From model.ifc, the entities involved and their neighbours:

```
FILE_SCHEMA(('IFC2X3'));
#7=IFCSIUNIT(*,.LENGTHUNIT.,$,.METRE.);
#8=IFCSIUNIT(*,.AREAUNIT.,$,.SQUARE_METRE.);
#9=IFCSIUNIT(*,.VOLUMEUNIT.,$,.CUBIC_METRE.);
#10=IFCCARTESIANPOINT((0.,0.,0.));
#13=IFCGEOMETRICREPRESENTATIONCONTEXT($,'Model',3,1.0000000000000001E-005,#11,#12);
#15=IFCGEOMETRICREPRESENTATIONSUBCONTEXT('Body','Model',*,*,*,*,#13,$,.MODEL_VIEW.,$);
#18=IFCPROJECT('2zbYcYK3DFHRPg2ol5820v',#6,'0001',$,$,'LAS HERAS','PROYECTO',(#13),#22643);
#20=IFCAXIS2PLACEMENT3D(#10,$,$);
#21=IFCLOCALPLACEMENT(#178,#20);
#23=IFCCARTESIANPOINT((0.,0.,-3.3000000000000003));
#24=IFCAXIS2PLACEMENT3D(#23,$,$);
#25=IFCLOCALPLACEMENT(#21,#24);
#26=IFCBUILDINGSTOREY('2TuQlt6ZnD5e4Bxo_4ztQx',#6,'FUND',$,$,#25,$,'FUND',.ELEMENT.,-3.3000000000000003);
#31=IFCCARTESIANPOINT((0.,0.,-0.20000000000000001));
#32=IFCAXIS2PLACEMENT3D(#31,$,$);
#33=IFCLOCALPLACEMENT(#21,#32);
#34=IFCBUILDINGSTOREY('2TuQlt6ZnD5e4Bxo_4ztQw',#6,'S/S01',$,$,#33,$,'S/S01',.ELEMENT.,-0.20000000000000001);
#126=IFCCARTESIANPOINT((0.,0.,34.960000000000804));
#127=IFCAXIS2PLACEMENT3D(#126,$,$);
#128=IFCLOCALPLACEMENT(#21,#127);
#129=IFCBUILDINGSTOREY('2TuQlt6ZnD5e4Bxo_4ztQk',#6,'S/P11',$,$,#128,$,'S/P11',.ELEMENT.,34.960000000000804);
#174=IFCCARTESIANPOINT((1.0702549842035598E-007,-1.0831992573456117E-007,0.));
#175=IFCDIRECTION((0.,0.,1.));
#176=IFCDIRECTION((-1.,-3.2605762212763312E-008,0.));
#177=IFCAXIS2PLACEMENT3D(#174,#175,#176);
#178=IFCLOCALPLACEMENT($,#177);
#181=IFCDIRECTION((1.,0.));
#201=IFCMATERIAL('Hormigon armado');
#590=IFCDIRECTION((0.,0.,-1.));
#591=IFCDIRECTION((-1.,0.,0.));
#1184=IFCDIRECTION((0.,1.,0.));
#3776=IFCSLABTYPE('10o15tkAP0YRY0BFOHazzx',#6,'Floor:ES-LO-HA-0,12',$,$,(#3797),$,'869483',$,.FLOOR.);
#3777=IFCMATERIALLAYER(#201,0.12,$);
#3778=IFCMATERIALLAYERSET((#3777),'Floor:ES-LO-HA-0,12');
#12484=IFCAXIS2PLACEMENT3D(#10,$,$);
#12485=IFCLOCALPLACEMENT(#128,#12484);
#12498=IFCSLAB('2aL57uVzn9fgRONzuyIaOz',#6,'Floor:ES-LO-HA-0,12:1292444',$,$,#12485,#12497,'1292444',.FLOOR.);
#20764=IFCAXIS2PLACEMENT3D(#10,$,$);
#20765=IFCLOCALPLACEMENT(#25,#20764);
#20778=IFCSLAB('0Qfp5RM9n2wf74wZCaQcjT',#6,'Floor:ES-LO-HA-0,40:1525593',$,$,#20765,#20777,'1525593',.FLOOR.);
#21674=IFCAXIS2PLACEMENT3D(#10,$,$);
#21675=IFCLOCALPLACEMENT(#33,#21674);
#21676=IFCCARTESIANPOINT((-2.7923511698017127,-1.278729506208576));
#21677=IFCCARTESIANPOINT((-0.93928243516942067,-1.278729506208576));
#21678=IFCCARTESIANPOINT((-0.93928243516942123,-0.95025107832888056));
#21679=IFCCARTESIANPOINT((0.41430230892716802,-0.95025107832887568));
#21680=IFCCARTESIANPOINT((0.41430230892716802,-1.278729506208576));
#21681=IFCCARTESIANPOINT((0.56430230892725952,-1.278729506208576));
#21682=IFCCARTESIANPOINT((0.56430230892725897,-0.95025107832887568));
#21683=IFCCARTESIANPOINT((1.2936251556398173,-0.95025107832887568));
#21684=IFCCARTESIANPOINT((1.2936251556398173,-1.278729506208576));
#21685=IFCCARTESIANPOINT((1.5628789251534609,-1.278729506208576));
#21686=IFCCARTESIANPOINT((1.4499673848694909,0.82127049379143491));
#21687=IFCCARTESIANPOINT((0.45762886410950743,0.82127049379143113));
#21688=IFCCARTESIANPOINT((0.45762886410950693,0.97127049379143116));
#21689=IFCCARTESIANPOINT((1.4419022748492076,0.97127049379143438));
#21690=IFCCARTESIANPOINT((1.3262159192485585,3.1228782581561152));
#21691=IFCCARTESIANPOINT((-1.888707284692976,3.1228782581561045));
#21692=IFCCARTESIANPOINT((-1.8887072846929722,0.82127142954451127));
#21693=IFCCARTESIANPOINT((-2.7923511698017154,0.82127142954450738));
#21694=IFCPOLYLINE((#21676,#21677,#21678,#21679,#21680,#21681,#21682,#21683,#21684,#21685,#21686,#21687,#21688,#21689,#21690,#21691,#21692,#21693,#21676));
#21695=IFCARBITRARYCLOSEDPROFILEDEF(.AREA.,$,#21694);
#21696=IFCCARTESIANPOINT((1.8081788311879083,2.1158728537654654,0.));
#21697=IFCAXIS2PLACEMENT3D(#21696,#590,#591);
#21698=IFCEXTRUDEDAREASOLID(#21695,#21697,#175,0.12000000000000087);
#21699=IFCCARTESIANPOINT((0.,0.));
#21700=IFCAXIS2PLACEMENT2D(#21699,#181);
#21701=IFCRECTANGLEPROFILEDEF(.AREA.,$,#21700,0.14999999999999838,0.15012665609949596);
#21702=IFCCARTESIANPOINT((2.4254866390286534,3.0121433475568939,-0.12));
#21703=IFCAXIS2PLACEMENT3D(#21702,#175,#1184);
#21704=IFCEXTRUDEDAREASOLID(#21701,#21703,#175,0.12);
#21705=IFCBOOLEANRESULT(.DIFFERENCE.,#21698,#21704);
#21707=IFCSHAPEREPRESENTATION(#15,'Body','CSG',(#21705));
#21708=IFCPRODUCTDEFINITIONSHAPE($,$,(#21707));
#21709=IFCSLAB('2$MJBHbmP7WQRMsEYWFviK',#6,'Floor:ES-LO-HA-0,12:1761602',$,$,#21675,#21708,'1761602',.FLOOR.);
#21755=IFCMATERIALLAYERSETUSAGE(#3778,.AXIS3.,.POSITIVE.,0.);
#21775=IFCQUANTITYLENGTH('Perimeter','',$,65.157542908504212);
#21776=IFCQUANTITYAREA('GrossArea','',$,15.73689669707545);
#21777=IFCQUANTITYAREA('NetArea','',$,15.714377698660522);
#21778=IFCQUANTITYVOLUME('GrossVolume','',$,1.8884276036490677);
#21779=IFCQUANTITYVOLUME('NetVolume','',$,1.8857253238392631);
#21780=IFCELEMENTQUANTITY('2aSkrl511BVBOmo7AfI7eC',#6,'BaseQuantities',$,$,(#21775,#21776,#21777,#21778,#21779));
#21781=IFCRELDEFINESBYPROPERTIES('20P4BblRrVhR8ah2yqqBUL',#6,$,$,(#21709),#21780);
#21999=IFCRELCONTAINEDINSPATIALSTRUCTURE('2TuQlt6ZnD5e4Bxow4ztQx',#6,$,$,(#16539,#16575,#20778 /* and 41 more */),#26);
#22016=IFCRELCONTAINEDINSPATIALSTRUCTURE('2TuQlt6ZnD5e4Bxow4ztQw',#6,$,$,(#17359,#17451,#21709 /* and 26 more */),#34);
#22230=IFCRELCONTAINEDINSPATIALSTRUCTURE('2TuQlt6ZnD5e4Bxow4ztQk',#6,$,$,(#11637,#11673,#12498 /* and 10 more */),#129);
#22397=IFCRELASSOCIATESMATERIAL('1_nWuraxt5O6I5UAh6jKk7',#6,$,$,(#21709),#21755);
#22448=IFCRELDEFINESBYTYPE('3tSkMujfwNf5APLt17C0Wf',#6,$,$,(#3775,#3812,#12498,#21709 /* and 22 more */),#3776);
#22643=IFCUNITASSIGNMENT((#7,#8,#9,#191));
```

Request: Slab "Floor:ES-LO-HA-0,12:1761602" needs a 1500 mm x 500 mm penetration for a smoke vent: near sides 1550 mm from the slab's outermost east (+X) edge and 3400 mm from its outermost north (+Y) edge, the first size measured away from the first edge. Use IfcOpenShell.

```python
import numpy as np
import ifcopenshell
import ifcopenshell.api.feature
import ifcopenshell.api.geometry
import ifcopenshell.api.pset
import ifcopenshell.api.root
import ifcopenshell.geom
import ifcopenshell.util.element
import ifcopenshell.util.placement
import ifcopenshell.util.representation
import ifcopenshell.util.shape
import ifcopenshell.util.unit

model = ifcopenshell.open("model.ifc")
unit_scale = ifcopenshell.util.unit.calculate_unit_scale(model)
area_scale = ifcopenshell.util.unit.calculate_unit_scale(model, "AREAUNIT")
volume_scale = ifcopenshell.util.unit.calculate_unit_scale(model, "VOLUMEUNIT")
settings = ifcopenshell.geom.settings()


def volume(element):
    """Net volume in cubic metres, openings subtracted."""
    shape = ifcopenshell.geom.create_shape(settings, element)
    return ifcopenshell.util.shape.get_volume(shape.geometry)


slab = model.by_guid("2$MJBHbmP7WQRMsEYWFviK")
before = volume(slab)

# Extent in the slab's own axes, in metres. The edges named are its -X and -Y sides.
slab_shape = ifcopenshell.geom.create_shape(settings, slab)
vertices = ifcopenshell.util.shape.get_vertices(slab_shape.geometry)
x_min, y_min, bottom = vertices.min(axis=0)
top = vertices[:, 2].max()

opening = ifcopenshell.api.root.create_entity(model, ifc_class="IfcOpeningElement", name="Smoke vent opening")
context = ifcopenshell.util.representation.get_context(model, "Model", "Body", "MODEL_VIEW")
width, depth = 1.5, 0.5
outline = [(0.0, 0.0), (width, 0.0), (width, depth), (0.0, depth), (0.0, 0.0)]
# Overshoot both faces by 50 mm so the cut is clean.
shape = ifcopenshell.api.geometry.add_slab_representation(
    model, context=context, depth=top - bottom + 0.1, polyline=outline
)
ifcopenshell.api.geometry.assign_representation(model, product=opening, representation=shape)

matrix = ifcopenshell.util.placement.get_local_placement(slab.ObjectPlacement)
matrix[:, 3] = matrix @ np.append(np.array([x_min + 1.55, y_min + 3.4, bottom - 0.05]) / unit_scale, 1.0)
ifcopenshell.api.geometry.edit_object_placement(model, product=opening, matrix=matrix, is_si=False)
ifcopenshell.api.feature.add_feature(model, feature=opening, element=slab)

after = volume(slab)

# Update the slab's stored quantities.
qto = model.by_id(ifcopenshell.util.element.get_pset(slab, "BaseQuantities", should_inherit=False)["id"])
ifcopenshell.api.pset.edit_qto(model, qto=qto, properties={
    "NetArea": after / (top - bottom) / area_scale,
    "NetVolume": after / volume_scale,
})

print(f"slab volume {before:.3f} -> {after:.3f} m3")

model.write("model_updated.ifc")
```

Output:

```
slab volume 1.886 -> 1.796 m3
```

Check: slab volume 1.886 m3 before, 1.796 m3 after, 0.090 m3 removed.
